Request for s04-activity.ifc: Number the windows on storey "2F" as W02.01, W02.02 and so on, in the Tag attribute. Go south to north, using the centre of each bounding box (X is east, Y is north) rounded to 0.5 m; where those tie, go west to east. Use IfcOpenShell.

First a look at what the model holds.

```python
import ifcopenshell
import ifcopenshell.util.element
import ifcopenshell.util.placement

model = ifcopenshell.open("s04-activity.ifc")
print(model.schema)
storey = next(s for s in model.by_type("IfcBuildingStorey") if s.Name == "2F")
windows = [e for e in ifcopenshell.util.element.get_decomposition(storey) if e.is_a("IfcWindow")]
for e in sorted(windows, key=lambda e: e.id()):
    origin = ifcopenshell.util.placement.get_local_placement(e.ObjectPlacement)[:3, 3]
    print(e.id(), e.Tag, e.Name, origin.round(2) + 0.0, sep=" | ")
```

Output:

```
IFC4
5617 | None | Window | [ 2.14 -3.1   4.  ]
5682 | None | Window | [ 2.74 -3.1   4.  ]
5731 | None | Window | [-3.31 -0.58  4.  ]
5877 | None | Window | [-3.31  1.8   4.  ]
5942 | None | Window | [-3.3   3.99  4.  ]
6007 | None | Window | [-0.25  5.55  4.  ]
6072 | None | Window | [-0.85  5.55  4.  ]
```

```python
import ifcopenshell
import ifcopenshell.geom
import ifcopenshell.util.element
import ifcopenshell.util.shape

model = ifcopenshell.open("s04-activity.ifc")
settings = ifcopenshell.geom.settings()
settings.set("use-world-coords", True)


def centre(element):
    shape = ifcopenshell.geom.create_shape(settings, element)
    return ifcopenshell.util.shape.get_bbox_centroid(shape.geometry)


storey = next(s for s in model.by_type("IfcBuildingStorey") if s.Name == "2F")
windows = [e for e in ifcopenshell.util.element.get_decomposition(storey) if e.is_a("IfcWindow")]

# Insertion points can sit at a corner or the storey origin, so sort by the geometry (in metres).
centres = {e: centre(e) for e in windows}
windows.sort(key=lambda e: (round(centres[e][1] / 0.5), centres[e][0]))

for i, e in enumerate(windows, start=1):
    number = f"W02.{i:02d}"
    e.Tag = number
    print(e.id(), number)

model.write("s04-activity_edited.ifc")
```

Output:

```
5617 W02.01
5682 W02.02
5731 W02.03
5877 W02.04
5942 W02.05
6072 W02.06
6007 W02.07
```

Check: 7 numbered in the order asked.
